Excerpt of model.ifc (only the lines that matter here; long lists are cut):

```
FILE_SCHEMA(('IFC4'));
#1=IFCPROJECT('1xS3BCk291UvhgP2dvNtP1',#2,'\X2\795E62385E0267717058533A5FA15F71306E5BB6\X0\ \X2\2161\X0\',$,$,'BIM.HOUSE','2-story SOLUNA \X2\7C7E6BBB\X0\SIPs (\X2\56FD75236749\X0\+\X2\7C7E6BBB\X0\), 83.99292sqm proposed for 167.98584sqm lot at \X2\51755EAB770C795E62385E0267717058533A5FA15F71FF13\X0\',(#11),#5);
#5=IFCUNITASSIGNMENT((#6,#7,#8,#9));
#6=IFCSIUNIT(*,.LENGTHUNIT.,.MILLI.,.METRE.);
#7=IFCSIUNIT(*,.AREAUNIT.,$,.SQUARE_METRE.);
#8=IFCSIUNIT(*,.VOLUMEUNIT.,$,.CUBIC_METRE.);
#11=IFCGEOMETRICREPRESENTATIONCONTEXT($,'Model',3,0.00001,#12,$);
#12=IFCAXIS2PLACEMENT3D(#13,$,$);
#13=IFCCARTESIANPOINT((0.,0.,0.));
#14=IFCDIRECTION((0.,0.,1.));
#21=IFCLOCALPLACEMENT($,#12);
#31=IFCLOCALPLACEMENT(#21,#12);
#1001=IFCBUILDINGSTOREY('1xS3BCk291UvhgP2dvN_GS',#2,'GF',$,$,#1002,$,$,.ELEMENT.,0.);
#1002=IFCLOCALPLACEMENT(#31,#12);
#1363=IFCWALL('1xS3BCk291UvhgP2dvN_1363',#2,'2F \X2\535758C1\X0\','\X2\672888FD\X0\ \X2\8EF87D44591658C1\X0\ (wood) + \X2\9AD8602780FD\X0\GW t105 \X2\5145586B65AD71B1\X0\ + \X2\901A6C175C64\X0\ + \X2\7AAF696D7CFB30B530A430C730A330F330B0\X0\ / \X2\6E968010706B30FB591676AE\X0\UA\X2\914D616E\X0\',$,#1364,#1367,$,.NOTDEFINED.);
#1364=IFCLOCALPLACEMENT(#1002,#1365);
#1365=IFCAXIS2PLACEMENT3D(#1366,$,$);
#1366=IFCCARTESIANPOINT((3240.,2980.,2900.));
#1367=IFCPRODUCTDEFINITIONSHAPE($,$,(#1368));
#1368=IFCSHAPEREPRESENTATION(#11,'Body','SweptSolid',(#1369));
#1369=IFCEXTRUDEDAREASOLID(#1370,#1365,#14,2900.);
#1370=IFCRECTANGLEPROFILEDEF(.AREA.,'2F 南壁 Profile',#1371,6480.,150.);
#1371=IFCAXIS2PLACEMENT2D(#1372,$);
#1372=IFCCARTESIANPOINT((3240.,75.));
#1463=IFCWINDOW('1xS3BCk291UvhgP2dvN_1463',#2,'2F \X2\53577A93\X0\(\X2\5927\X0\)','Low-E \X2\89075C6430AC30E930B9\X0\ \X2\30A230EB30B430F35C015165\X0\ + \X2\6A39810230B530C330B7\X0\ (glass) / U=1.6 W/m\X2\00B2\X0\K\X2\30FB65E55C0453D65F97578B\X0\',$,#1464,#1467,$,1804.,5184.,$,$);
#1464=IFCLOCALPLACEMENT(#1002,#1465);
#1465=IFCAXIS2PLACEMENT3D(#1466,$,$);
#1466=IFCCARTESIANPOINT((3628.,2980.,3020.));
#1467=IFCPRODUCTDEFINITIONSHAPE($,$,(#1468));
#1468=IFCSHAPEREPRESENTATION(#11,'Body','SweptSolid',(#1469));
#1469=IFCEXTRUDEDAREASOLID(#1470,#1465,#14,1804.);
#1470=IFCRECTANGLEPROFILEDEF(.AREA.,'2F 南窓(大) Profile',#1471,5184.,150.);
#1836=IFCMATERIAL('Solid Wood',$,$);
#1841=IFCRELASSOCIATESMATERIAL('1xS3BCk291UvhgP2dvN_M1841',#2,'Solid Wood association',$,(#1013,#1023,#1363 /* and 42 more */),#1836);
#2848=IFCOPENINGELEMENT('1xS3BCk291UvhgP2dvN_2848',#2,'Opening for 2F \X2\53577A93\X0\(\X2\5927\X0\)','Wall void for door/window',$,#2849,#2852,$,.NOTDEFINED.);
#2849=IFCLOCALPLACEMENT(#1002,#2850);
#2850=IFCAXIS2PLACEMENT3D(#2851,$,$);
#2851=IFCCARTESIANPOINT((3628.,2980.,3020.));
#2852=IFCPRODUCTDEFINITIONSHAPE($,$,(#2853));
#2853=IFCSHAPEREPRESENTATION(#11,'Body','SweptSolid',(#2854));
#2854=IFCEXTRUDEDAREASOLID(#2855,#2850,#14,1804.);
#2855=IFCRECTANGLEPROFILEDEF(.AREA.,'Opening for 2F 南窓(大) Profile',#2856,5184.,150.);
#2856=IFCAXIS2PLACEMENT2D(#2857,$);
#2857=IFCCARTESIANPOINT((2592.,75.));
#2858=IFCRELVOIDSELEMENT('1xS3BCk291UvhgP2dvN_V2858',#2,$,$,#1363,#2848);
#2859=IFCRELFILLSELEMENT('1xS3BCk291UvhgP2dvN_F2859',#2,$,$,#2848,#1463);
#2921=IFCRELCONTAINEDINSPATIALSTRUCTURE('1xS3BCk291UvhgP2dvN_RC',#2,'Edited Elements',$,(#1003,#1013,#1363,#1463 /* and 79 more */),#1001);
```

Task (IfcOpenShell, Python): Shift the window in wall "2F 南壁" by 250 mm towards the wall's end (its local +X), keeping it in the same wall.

```python
import ifcopenshell
import ifcopenshell.api.geometry
import ifcopenshell.util.placement

model = ifcopenshell.open("model.ifc")

window = model.by_guid("1xS3BCk291UvhgP2dvN_1463")
opening = window.FillsVoids[0].RelatingOpeningElement
wall = opening.VoidsElements[0].RelatingBuildingElement

wall_matrix = ifcopenshell.util.placement.get_local_placement(wall.ObjectPlacement)
shift = wall_matrix[:3, 0] * 250.0
before = ifcopenshell.util.placement.get_local_placement(window.ObjectPlacement)[:3, 3].copy()

# The window is not placed relative to its opening, so move both.
for product in (opening, window):
    matrix = ifcopenshell.util.placement.get_local_placement(product.ObjectPlacement)
    matrix[:3, 3] += shift
    ifcopenshell.api.geometry.edit_object_placement(model, product=product, matrix=matrix, is_si=False)

after = ifcopenshell.util.placement.get_local_placement(window.ObjectPlacement)[:3, 3]
print("window moved by", (after - before).round(3) + 0.0)

model.write("model_edited.ifc")
```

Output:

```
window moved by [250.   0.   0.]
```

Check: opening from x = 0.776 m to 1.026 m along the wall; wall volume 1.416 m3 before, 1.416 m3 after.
